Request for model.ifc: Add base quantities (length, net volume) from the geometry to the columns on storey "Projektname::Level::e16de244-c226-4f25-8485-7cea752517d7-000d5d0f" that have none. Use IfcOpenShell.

First a look at what the model holds.

```python
import ifcopenshell
import ifcopenshell.util.element
import ifcopenshell.util.unit

model = ifcopenshell.open("model.ifc")
print(model.schema)
for unit_type in ("LENGTHUNIT", "AREAUNIT", "VOLUMEUNIT"):
    print(unit_type, ifcopenshell.util.unit.calculate_unit_scale(model, unit_type))
storey = next(s for s in model.by_type("IfcBuildingStorey") if s.Name == "Projektname::Level::e16de244-c226-4f25-8485-7cea752517d7-000d5d0f")
columns = [e for e in ifcopenshell.util.element.get_decomposition(storey) if e.is_a("IfcColumn")]
for e in sorted(columns, key=lambda e: e.id()):
    print(e.id(), e.is_a(), e.Name, list(ifcopenshell.util.element.get_psets(e, qtos_only=True)), sep=" | ")
```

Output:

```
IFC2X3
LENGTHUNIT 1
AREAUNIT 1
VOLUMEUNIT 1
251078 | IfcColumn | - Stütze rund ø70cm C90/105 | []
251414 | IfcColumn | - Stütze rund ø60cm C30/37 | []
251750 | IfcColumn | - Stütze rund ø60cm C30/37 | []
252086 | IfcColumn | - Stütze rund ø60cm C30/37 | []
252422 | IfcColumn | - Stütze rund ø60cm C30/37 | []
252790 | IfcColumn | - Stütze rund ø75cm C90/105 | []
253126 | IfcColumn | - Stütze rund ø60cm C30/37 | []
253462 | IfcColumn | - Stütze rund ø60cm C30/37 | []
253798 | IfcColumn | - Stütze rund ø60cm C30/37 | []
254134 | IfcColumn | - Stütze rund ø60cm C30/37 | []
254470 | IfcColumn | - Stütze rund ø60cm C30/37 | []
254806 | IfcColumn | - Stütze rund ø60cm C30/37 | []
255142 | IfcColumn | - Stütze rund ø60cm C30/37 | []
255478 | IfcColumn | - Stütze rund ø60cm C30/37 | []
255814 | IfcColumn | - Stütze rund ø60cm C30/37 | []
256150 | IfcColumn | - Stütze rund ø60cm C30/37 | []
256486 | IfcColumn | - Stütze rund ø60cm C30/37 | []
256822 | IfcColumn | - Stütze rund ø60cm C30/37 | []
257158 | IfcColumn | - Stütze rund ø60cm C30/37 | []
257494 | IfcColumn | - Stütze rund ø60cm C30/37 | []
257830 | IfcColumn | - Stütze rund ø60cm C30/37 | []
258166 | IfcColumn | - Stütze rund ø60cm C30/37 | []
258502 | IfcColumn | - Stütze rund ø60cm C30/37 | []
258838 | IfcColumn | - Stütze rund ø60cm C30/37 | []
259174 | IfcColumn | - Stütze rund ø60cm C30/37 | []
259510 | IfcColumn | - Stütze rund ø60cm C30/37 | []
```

```python
import ifcopenshell
import ifcopenshell.api.pset
import ifcopenshell.geom
import ifcopenshell.util.element
import ifcopenshell.util.shape
import ifcopenshell.util.unit

model = ifcopenshell.open("model.ifc")
unit_scale = ifcopenshell.util.unit.calculate_unit_scale(model)
volume_scale = ifcopenshell.util.unit.calculate_unit_scale(model, "VOLUMEUNIT")
settings = ifcopenshell.geom.settings()

storey = next(s for s in model.by_type("IfcBuildingStorey") if s.Name == "Projektname::Level::e16de244-c226-4f25-8485-7cea752517d7-000d5d0f")
columns = [e for e in ifcopenshell.util.element.get_decomposition(storey) if e.is_a("IfcColumn")]

for e in sorted(columns, key=lambda e: e.id()):
    if ifcopenshell.util.element.get_psets(e, qtos_only=True, should_inherit=False):
        continue
    # Geometry comes back in metres, in the element's own axes.
    shape = ifcopenshell.geom.create_shape(settings, e)
    values = {
        "Length": ifcopenshell.util.shape.get_z(shape.geometry) / unit_scale,
        "NetVolume": ifcopenshell.util.shape.get_volume(shape.geometry) / volume_scale,
    }
    qto = ifcopenshell.api.pset.add_qto(model, product=e, name="BaseQuantities")
    ifcopenshell.api.pset.edit_qto(model, qto=qto, properties=values)
    print(e.id(), {k: round(v, 3) for k, v in values.items()})

model.write("model_edited.ifc")
```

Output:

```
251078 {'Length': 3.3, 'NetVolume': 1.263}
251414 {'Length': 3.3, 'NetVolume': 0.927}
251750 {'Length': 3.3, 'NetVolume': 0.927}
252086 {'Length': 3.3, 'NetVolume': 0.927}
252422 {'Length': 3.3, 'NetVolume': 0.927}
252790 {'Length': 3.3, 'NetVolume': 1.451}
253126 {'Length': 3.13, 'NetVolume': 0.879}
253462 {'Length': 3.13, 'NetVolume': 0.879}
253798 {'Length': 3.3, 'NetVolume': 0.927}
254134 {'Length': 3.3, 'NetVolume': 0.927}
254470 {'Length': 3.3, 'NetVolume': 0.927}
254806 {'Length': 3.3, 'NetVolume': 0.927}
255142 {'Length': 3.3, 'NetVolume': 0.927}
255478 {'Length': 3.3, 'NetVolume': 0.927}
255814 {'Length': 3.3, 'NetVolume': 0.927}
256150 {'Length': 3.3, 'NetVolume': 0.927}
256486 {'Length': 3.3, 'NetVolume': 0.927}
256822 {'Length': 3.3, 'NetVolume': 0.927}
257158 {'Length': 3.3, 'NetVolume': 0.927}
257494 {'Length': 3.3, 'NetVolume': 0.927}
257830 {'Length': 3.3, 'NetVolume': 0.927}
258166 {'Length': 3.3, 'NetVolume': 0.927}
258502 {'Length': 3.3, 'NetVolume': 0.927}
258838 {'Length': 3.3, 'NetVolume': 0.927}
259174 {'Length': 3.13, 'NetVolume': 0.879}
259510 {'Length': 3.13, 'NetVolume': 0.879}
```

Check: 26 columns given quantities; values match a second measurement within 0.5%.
